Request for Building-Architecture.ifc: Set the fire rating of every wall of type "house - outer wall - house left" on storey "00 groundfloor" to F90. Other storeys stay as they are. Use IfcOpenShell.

First a look at what the model holds.

```python
import ifcopenshell
import ifcopenshell.util.element

model = ifcopenshell.open("Building-Architecture.ifc")
print(model.schema)
storey = next(s for s in model.by_type("IfcBuildingStorey") if s.Name == "00 groundfloor")
walls = [e for e in ifcopenshell.util.element.get_decomposition(storey) if e.is_a("IfcWall")]
seen = {}
for e in walls:
    element_type = ifcopenshell.util.element.get_type(e)
    key = (element_type.Name if element_type != e and element_type else None, ifcopenshell.util.element.get_pset(e, "Pset_WallCommon", "FireRating"))
    seen[key] = seen.get(key, 0) + 1
for (name, value), count in sorted(seen.items(), key=str):
    print(count, "x", name, "|", value)
```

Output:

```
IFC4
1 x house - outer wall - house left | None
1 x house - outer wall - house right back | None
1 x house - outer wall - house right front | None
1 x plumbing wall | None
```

```python
import ifcopenshell
import ifcopenshell.api.pset
import ifcopenshell.util.element

model = ifcopenshell.open("Building-Architecture.ifc")

storey = next(s for s in model.by_type("IfcBuildingStorey") if s.Name == "00 groundfloor")
walls = [e for e in ifcopenshell.util.element.get_decomposition(storey) if e.is_a("IfcWall")]

count = 0
for e in walls:
    element_type = ifcopenshell.util.element.get_type(e)
    if element_type in (None, e) or element_type.Name != "house - outer wall - house left":
        continue
    # add_pset returns the element's existing set when there is one.
    pset = ifcopenshell.api.pset.add_pset(model, product=e, name="Pset_WallCommon")
    ifcopenshell.api.pset.edit_pset(model, pset=pset, properties={"FireRating": "F90"})
    count += 1

print(count, "walls updated")

model.write("Building-Architecture_edited.ifc")
```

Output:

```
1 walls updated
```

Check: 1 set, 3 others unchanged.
